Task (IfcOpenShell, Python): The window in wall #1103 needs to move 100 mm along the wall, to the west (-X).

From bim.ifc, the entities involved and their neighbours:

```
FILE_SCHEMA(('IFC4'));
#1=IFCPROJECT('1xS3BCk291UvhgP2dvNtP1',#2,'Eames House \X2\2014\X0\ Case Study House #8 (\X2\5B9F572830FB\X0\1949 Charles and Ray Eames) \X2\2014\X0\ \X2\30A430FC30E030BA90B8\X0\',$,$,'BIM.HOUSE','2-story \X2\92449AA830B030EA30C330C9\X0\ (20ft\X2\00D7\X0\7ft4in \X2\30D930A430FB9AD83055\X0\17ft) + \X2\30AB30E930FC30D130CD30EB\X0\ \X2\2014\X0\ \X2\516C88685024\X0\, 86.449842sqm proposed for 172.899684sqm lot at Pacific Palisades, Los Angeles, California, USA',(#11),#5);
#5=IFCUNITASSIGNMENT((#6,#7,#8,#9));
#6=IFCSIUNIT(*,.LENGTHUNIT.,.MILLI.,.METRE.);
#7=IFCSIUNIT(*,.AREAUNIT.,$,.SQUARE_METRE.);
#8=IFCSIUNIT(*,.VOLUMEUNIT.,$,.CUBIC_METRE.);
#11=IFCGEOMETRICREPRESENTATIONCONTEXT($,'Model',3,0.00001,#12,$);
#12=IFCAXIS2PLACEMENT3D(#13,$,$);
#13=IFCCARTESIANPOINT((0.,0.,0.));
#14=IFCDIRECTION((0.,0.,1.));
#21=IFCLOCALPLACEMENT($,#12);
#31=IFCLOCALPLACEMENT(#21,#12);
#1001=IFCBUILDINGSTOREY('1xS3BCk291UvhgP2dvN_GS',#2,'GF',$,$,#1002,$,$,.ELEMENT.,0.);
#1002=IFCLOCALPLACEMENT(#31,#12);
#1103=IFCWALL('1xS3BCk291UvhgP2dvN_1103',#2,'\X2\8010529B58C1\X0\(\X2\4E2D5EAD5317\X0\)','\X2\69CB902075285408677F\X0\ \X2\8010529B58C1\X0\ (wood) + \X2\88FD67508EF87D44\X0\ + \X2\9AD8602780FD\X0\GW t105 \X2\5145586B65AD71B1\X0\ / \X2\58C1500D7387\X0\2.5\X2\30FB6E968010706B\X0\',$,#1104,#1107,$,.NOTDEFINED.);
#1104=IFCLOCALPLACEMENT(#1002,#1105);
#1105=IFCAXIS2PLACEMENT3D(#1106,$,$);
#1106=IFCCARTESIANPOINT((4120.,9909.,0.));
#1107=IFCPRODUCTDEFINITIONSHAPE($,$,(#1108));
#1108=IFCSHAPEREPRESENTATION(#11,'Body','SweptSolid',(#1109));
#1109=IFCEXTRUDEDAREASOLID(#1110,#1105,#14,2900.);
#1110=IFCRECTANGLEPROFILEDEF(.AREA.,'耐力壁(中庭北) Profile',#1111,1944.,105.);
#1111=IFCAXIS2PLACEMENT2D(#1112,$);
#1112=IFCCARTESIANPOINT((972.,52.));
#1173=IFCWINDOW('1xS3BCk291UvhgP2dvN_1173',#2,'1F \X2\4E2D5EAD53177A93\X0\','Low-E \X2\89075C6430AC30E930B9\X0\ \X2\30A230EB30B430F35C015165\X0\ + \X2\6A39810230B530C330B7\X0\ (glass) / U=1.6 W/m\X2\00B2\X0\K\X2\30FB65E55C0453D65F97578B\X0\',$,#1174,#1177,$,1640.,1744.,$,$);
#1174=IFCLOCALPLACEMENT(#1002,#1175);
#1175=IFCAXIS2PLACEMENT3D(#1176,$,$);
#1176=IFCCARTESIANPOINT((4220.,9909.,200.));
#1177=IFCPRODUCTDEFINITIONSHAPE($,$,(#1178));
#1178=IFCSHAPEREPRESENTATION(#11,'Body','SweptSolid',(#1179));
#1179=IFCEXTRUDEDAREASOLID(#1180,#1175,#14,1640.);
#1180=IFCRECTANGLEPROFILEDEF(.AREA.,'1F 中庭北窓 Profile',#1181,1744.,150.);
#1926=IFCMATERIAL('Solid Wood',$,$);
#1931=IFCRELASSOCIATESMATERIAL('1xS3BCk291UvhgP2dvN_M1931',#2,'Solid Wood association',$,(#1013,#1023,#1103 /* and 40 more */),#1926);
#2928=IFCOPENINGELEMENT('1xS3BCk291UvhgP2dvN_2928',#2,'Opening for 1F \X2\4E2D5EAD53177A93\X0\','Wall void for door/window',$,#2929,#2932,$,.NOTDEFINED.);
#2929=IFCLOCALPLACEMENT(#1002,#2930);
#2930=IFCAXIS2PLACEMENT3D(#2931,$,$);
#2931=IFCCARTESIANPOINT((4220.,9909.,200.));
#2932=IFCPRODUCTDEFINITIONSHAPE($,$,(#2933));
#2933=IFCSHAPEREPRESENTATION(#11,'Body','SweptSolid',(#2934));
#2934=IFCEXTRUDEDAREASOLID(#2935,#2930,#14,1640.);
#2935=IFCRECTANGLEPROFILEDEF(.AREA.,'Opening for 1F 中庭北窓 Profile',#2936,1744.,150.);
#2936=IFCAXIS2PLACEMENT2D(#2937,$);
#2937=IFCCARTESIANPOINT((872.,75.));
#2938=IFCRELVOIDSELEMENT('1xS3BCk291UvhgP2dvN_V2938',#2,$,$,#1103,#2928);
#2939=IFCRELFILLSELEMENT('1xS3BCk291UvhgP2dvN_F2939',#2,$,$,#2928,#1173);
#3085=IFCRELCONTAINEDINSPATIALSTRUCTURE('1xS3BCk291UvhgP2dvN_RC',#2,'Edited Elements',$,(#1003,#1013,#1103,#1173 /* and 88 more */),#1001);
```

```python
import ifcopenshell
import ifcopenshell.api.geometry
import ifcopenshell.util.placement
import ifcopenshell.util.unit

model = ifcopenshell.open("bim.ifc")
unit_scale = ifcopenshell.util.unit.calculate_unit_scale(model)

window = model.by_guid("1xS3BCk291UvhgP2dvN_1173")
opening = window.FillsVoids[0].RelatingOpeningElement
wall = opening.VoidsElements[0].RelatingBuildingElement

wall_matrix = ifcopenshell.util.placement.get_local_placement(wall.ObjectPlacement)
shift = wall_matrix[:3, 0] * -0.1 / unit_scale
before = ifcopenshell.util.placement.get_local_placement(window.ObjectPlacement)[:3, 3].copy()

# The window is not placed relative to its opening, so move both.
for product in (opening, window):
    matrix = ifcopenshell.util.placement.get_local_placement(product.ObjectPlacement)
    matrix[:3, 3] += shift
    ifcopenshell.api.geometry.edit_object_placement(model, product=product, matrix=matrix, is_si=False)

after = ifcopenshell.util.placement.get_local_placement(window.ObjectPlacement)[:3, 3]
print("window moved by", (after - before).round(3) + 0.0)

model.write("bim_edited.ifc")
```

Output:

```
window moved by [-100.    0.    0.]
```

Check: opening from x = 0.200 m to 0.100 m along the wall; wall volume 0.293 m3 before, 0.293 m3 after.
